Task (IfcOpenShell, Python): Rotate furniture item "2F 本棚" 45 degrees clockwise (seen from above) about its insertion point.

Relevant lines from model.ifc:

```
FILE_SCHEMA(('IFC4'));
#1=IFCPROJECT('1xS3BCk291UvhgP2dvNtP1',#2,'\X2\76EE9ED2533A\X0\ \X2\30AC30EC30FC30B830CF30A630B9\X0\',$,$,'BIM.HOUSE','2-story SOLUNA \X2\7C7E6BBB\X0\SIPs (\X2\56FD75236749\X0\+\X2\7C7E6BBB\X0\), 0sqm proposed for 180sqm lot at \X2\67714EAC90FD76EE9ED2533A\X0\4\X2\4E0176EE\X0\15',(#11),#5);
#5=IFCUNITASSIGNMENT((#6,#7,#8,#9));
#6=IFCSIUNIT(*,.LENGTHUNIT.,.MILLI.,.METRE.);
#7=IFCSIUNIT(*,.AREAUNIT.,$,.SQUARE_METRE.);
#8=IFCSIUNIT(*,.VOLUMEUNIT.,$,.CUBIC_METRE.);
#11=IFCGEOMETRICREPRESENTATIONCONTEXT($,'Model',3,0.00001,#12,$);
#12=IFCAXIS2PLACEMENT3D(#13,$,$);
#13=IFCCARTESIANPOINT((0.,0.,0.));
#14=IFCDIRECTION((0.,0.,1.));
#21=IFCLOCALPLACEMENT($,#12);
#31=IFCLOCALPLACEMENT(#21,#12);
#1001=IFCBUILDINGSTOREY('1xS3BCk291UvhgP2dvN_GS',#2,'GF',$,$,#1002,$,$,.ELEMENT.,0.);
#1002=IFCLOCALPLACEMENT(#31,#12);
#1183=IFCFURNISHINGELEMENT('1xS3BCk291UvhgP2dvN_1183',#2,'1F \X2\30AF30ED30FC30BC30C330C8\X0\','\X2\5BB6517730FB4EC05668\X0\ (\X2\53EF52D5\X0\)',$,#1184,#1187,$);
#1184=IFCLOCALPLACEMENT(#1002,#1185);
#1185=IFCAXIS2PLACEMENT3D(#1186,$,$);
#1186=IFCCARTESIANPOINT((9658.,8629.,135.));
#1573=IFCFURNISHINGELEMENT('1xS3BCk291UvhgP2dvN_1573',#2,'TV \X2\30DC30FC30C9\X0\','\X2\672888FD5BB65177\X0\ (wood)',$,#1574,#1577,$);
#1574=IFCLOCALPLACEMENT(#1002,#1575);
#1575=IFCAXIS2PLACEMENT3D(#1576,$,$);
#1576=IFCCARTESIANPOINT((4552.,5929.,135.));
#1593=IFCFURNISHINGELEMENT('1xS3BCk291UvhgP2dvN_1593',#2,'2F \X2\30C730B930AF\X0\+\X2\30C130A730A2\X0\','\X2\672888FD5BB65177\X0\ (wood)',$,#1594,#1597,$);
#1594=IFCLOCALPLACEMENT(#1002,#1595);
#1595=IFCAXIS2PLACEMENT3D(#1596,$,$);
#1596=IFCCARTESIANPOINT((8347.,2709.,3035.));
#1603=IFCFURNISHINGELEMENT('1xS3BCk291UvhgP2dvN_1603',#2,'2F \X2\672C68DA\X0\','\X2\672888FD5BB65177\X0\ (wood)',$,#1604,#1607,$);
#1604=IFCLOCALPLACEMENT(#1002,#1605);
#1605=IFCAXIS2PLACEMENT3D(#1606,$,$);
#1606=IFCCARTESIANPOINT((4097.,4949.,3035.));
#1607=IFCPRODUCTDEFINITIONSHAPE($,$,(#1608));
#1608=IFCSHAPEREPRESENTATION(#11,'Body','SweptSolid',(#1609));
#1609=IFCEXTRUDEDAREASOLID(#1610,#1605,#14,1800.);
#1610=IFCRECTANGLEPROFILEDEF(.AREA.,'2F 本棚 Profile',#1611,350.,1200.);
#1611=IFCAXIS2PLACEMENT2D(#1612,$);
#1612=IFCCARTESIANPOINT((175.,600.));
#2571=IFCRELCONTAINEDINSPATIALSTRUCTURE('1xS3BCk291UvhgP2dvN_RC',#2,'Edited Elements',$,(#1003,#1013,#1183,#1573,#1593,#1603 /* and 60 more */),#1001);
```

```python
import ifcopenshell
import ifcopenshell.api.geometry
import ifcopenshell.util.placement

model = ifcopenshell.open("model.ifc")

item = model.by_guid("1xS3BCk291UvhgP2dvN_1603")
matrix = ifcopenshell.util.placement.get_local_placement(item.ObjectPlacement)
matrix = matrix @ ifcopenshell.util.placement.rotation(-45, "Z")
ifcopenshell.api.geometry.edit_object_placement(model, product=item, matrix=matrix, is_si=False)

print(ifcopenshell.util.placement.get_local_placement(item.ObjectPlacement).round(3) + 0.0)

model.write("model-out.ifc")
```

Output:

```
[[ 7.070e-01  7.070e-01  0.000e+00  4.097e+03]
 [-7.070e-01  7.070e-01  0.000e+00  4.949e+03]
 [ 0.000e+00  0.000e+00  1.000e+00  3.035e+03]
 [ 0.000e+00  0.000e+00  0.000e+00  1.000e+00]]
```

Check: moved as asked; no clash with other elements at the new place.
